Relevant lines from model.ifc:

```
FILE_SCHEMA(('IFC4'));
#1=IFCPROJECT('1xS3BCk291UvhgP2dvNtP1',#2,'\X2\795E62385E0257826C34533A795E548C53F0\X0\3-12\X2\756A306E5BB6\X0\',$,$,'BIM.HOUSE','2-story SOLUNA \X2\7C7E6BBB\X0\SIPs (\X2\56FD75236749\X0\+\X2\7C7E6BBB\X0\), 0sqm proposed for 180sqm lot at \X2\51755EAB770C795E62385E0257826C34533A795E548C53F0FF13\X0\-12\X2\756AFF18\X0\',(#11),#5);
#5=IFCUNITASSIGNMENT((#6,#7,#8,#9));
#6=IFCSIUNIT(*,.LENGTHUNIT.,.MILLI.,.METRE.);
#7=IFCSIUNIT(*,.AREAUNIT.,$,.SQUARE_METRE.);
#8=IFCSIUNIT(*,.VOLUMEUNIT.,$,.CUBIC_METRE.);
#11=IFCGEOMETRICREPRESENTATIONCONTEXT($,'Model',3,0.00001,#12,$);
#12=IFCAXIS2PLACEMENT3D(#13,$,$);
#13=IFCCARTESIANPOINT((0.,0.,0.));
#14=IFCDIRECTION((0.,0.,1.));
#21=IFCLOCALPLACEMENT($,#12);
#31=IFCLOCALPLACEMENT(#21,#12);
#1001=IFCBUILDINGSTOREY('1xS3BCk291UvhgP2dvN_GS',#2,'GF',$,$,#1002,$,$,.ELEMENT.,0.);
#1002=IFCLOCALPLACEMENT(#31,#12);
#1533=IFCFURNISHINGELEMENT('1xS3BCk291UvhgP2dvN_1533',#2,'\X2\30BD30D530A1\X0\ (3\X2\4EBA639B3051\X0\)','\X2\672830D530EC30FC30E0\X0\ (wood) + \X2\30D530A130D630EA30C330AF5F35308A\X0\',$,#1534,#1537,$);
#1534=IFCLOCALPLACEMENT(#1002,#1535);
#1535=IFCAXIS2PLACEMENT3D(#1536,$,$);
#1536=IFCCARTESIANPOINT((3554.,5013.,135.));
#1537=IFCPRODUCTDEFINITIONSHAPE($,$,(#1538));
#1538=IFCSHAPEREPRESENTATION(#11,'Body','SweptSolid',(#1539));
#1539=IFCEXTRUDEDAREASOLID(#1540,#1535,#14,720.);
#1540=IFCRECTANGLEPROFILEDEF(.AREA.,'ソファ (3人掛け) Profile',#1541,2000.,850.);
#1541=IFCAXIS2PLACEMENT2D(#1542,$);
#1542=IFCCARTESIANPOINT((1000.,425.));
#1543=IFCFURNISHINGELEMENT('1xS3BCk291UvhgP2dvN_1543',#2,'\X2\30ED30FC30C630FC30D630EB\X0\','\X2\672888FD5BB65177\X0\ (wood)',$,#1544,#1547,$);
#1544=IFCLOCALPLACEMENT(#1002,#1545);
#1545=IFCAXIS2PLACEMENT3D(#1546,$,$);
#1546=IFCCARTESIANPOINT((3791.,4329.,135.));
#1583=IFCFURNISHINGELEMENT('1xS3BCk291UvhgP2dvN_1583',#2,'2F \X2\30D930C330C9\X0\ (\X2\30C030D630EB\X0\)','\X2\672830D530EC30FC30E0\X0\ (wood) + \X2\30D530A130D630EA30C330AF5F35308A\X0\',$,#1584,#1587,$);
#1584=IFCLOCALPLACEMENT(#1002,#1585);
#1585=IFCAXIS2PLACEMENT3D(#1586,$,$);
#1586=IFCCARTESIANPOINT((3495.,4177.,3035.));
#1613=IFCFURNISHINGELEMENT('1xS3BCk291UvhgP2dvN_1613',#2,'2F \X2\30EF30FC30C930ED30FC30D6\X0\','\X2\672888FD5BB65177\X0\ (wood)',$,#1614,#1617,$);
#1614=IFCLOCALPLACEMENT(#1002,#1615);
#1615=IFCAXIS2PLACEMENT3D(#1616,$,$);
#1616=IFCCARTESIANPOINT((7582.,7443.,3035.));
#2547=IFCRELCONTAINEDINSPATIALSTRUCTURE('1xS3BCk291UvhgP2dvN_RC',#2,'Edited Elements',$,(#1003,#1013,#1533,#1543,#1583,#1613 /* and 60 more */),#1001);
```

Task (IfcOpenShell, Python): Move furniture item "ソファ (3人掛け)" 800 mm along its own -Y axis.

```python
import ifcopenshell
import ifcopenshell.api.geometry
import ifcopenshell.util.placement

model = ifcopenshell.open("model.ifc")

item = model.by_guid("1xS3BCk291UvhgP2dvN_1533")
matrix = ifcopenshell.util.placement.get_local_placement(item.ObjectPlacement)
matrix[:3, 3] -= matrix[:3, 1] * 800.0
ifcopenshell.api.geometry.edit_object_placement(model, product=item, matrix=matrix, is_si=False)

print(ifcopenshell.util.placement.get_local_placement(item.ObjectPlacement).round(3) + 0.0)

model.write("model_v2.ifc")
```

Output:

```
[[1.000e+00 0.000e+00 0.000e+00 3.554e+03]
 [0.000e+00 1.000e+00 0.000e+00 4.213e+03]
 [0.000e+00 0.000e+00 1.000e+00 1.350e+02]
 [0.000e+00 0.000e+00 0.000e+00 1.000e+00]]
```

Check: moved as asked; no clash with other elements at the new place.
